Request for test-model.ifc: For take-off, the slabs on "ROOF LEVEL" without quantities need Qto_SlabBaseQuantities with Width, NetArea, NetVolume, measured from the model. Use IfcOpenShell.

First a look at what the model holds.

```python
import ifcopenshell
import ifcopenshell.util.element
import ifcopenshell.util.unit

model = ifcopenshell.open("test-model.ifc")
print(model.schema)
for unit_type in ("LENGTHUNIT", "AREAUNIT", "VOLUMEUNIT"):
    print(unit_type, ifcopenshell.util.unit.calculate_unit_scale(model, unit_type))
storey = next(s for s in model.by_type("IfcBuildingStorey") if s.Name == "ROOF LEVEL")
slabs = [e for e in ifcopenshell.util.element.get_decomposition(storey) if e.is_a("IfcSlab")]
for e in sorted(slabs, key=lambda e: e.id()):
    print(e.id(), e.is_a(), e.Name, list(ifcopenshell.util.element.get_psets(e, qtos_only=True)), sep=" | ")
```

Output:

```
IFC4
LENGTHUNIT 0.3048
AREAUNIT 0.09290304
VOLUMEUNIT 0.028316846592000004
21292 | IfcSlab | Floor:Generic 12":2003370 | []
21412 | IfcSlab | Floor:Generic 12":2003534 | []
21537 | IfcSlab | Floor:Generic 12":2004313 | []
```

```python
import ifcopenshell
import ifcopenshell.api.pset
import ifcopenshell.geom
import ifcopenshell.util.element
import ifcopenshell.util.shape
import ifcopenshell.util.unit

model = ifcopenshell.open("test-model.ifc")
unit_scale = ifcopenshell.util.unit.calculate_unit_scale(model)
area_scale = ifcopenshell.util.unit.calculate_unit_scale(model, "AREAUNIT")
volume_scale = ifcopenshell.util.unit.calculate_unit_scale(model, "VOLUMEUNIT")
settings = ifcopenshell.geom.settings()

storey = next(s for s in model.by_type("IfcBuildingStorey") if s.Name == "ROOF LEVEL")
slabs = [e for e in ifcopenshell.util.element.get_decomposition(storey) if e.is_a("IfcSlab")]

for e in sorted(slabs, key=lambda e: e.id()):
    if ifcopenshell.util.element.get_psets(e, qtos_only=True, should_inherit=False):
        continue
    # Geometry comes back in metres, in the element's own axes.
    shape = ifcopenshell.geom.create_shape(settings, e)
    values = {
        "Width": ifcopenshell.util.shape.get_z(shape.geometry) / unit_scale,
        "NetArea": ifcopenshell.util.shape.get_footprint_area(shape.geometry) / area_scale,
        "NetVolume": ifcopenshell.util.shape.get_volume(shape.geometry) / volume_scale,
    }
    qto = ifcopenshell.api.pset.add_qto(model, product=e, name="Qto_SlabBaseQuantities")
    ifcopenshell.api.pset.edit_qto(model, qto=qto, properties=values)
    print(e.id(), {k: round(v, 3) for k, v in values.items()})

model.write("test-model_v2.ifc")
```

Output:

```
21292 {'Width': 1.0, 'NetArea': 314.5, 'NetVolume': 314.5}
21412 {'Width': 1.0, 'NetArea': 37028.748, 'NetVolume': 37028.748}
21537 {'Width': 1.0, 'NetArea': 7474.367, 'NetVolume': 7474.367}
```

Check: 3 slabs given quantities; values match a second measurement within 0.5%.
